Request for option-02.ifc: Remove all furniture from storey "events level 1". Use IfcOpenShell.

First a look at what the model holds.

```python
import ifcopenshell
import ifcopenshell.util.element

model = ifcopenshell.open("option-02.ifc")
print(model.schema)
storey = next(s for s in model.by_type("IfcBuildingStorey") if s.Name == "events level 1")
furniture = [e for e in ifcopenshell.util.element.get_decomposition(storey) if e.is_a("IfcFurnishingElement")]
seen = {}
for e in furniture:
    element_type = ifcopenshell.util.element.get_type(e)
    name = element_type.Name if element_type not in (None, e) else None
    seen[name] = seen.get(name, 0) + 1
for name, count in sorted(seen.items(), key=str):
    print(count, "x", name)
```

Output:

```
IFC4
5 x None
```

```python
import ifcopenshell
import ifcopenshell.api.root
import ifcopenshell.util.element

model = ifcopenshell.open("option-02.ifc")

storey = next(s for s in model.by_type("IfcBuildingStorey") if s.Name == "events level 1")
furniture = [e for e in ifcopenshell.util.element.get_decomposition(storey) if e.is_a("IfcFurnishingElement")]

for e in furniture:
    ifcopenshell.api.root.remove_product(model, product=e)
print(len(furniture), "removed")

model.write("option-02_updated.ifc")
```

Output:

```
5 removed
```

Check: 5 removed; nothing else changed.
